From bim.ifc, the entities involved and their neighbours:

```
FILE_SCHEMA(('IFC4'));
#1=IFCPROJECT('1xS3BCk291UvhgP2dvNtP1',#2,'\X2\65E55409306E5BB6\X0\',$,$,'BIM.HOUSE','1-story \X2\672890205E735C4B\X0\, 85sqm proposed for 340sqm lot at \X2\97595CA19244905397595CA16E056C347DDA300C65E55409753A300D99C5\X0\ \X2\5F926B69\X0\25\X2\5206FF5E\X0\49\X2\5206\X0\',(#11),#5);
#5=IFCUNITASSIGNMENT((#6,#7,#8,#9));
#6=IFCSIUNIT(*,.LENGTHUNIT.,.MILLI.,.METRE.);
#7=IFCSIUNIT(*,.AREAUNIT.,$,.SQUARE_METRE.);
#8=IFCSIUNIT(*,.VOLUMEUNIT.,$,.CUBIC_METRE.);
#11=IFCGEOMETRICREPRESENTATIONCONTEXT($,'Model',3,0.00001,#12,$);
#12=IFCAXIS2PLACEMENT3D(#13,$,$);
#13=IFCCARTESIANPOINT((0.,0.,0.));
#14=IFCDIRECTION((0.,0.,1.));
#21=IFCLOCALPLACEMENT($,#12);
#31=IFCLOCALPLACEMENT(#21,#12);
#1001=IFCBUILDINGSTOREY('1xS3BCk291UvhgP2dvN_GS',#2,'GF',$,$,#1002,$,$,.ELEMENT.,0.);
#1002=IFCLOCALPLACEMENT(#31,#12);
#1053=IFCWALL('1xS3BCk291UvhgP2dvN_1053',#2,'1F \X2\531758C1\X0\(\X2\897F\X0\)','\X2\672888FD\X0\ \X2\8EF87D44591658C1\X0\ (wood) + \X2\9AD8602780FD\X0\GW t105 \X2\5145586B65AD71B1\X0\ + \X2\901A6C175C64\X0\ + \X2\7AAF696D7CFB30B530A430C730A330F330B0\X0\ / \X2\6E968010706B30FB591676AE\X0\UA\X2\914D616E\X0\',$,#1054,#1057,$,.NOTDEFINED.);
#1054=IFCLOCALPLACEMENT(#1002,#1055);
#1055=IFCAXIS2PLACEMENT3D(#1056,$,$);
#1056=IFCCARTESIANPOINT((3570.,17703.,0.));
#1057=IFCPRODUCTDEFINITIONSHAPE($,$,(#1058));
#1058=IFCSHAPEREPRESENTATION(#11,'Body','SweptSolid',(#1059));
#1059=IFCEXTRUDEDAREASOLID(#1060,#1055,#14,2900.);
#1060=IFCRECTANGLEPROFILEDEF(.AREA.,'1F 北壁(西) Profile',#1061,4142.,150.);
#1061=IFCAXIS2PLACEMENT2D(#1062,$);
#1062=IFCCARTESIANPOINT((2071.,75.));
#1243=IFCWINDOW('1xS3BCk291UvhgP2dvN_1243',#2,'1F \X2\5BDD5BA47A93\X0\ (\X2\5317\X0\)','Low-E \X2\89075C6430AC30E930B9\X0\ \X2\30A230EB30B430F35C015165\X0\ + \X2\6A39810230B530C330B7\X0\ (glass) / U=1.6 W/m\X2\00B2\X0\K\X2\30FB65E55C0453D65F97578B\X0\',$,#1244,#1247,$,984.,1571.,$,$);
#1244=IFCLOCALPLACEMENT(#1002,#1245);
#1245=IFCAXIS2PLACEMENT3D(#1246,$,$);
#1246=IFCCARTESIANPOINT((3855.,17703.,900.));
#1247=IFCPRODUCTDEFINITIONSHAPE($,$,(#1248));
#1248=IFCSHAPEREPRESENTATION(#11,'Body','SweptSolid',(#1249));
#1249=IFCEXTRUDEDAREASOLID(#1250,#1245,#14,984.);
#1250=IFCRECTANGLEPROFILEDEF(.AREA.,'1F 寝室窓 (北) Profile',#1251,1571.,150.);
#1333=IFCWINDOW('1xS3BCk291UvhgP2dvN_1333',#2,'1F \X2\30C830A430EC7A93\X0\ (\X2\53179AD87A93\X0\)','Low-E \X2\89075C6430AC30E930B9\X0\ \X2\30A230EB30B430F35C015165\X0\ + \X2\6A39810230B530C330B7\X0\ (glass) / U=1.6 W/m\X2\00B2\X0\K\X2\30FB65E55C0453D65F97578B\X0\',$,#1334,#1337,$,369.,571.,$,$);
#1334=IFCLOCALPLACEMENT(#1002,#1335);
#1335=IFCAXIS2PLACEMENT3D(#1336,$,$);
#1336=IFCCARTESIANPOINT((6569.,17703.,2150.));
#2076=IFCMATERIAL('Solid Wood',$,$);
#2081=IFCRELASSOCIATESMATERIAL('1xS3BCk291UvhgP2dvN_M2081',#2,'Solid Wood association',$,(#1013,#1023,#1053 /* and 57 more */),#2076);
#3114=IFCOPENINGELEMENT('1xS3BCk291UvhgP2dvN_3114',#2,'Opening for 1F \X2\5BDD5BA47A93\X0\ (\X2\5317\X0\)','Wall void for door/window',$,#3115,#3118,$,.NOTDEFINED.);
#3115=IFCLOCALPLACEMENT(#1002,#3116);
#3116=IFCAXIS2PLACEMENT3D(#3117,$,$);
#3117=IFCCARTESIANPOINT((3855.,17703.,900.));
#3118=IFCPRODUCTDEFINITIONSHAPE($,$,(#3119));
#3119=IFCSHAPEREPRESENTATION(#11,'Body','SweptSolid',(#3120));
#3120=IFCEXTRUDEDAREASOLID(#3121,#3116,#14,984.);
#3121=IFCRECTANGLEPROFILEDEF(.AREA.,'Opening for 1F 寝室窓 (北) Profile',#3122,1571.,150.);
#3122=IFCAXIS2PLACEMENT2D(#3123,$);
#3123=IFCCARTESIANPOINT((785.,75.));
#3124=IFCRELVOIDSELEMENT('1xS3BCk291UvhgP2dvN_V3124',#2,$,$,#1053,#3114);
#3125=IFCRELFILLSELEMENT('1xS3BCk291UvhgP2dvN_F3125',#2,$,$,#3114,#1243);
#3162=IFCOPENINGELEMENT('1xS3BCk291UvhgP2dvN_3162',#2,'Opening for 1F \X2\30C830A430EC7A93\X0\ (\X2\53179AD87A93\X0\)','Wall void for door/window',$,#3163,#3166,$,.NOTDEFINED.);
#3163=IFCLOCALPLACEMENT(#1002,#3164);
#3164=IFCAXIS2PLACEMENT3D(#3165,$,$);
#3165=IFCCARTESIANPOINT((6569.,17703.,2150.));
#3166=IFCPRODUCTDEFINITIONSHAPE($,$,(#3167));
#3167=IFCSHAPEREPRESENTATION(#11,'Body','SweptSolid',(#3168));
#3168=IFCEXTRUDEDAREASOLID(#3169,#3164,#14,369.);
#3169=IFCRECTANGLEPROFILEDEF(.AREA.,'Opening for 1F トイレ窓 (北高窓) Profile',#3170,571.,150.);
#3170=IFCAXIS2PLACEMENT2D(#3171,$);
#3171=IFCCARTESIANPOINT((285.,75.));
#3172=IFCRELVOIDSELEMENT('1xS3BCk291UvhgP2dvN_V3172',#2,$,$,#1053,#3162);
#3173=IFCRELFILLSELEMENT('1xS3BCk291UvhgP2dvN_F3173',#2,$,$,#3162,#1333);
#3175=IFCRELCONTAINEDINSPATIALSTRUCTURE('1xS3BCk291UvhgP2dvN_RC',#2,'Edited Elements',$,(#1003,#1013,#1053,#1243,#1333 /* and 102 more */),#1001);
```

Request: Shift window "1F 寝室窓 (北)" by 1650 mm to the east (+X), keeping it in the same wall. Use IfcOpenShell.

```python
import ifcopenshell
import ifcopenshell.api.geometry
import ifcopenshell.util.placement

model = ifcopenshell.open("bim.ifc")

window = model.by_id(1243)
opening = window.FillsVoids[0].RelatingOpeningElement
wall = opening.VoidsElements[0].RelatingBuildingElement

wall_matrix = ifcopenshell.util.placement.get_local_placement(wall.ObjectPlacement)
shift = wall_matrix[:3, 0] * 1650.0
before = ifcopenshell.util.placement.get_local_placement(window.ObjectPlacement)[:3, 3].copy()

# The window is not placed relative to its opening, so move both.
for product in (opening, window):
    matrix = ifcopenshell.util.placement.get_local_placement(product.ObjectPlacement)
    matrix[:3, 3] += shift
    ifcopenshell.api.geometry.edit_object_placement(model, product=product, matrix=matrix, is_si=False)

after = ifcopenshell.util.placement.get_local_placement(window.ObjectPlacement)[:3, 3]
print("window moved by", (after - before).round(3) + 0.0)

model.write("bim_rev.ifc")
```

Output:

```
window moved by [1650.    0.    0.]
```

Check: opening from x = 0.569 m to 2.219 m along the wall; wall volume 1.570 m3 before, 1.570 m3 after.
